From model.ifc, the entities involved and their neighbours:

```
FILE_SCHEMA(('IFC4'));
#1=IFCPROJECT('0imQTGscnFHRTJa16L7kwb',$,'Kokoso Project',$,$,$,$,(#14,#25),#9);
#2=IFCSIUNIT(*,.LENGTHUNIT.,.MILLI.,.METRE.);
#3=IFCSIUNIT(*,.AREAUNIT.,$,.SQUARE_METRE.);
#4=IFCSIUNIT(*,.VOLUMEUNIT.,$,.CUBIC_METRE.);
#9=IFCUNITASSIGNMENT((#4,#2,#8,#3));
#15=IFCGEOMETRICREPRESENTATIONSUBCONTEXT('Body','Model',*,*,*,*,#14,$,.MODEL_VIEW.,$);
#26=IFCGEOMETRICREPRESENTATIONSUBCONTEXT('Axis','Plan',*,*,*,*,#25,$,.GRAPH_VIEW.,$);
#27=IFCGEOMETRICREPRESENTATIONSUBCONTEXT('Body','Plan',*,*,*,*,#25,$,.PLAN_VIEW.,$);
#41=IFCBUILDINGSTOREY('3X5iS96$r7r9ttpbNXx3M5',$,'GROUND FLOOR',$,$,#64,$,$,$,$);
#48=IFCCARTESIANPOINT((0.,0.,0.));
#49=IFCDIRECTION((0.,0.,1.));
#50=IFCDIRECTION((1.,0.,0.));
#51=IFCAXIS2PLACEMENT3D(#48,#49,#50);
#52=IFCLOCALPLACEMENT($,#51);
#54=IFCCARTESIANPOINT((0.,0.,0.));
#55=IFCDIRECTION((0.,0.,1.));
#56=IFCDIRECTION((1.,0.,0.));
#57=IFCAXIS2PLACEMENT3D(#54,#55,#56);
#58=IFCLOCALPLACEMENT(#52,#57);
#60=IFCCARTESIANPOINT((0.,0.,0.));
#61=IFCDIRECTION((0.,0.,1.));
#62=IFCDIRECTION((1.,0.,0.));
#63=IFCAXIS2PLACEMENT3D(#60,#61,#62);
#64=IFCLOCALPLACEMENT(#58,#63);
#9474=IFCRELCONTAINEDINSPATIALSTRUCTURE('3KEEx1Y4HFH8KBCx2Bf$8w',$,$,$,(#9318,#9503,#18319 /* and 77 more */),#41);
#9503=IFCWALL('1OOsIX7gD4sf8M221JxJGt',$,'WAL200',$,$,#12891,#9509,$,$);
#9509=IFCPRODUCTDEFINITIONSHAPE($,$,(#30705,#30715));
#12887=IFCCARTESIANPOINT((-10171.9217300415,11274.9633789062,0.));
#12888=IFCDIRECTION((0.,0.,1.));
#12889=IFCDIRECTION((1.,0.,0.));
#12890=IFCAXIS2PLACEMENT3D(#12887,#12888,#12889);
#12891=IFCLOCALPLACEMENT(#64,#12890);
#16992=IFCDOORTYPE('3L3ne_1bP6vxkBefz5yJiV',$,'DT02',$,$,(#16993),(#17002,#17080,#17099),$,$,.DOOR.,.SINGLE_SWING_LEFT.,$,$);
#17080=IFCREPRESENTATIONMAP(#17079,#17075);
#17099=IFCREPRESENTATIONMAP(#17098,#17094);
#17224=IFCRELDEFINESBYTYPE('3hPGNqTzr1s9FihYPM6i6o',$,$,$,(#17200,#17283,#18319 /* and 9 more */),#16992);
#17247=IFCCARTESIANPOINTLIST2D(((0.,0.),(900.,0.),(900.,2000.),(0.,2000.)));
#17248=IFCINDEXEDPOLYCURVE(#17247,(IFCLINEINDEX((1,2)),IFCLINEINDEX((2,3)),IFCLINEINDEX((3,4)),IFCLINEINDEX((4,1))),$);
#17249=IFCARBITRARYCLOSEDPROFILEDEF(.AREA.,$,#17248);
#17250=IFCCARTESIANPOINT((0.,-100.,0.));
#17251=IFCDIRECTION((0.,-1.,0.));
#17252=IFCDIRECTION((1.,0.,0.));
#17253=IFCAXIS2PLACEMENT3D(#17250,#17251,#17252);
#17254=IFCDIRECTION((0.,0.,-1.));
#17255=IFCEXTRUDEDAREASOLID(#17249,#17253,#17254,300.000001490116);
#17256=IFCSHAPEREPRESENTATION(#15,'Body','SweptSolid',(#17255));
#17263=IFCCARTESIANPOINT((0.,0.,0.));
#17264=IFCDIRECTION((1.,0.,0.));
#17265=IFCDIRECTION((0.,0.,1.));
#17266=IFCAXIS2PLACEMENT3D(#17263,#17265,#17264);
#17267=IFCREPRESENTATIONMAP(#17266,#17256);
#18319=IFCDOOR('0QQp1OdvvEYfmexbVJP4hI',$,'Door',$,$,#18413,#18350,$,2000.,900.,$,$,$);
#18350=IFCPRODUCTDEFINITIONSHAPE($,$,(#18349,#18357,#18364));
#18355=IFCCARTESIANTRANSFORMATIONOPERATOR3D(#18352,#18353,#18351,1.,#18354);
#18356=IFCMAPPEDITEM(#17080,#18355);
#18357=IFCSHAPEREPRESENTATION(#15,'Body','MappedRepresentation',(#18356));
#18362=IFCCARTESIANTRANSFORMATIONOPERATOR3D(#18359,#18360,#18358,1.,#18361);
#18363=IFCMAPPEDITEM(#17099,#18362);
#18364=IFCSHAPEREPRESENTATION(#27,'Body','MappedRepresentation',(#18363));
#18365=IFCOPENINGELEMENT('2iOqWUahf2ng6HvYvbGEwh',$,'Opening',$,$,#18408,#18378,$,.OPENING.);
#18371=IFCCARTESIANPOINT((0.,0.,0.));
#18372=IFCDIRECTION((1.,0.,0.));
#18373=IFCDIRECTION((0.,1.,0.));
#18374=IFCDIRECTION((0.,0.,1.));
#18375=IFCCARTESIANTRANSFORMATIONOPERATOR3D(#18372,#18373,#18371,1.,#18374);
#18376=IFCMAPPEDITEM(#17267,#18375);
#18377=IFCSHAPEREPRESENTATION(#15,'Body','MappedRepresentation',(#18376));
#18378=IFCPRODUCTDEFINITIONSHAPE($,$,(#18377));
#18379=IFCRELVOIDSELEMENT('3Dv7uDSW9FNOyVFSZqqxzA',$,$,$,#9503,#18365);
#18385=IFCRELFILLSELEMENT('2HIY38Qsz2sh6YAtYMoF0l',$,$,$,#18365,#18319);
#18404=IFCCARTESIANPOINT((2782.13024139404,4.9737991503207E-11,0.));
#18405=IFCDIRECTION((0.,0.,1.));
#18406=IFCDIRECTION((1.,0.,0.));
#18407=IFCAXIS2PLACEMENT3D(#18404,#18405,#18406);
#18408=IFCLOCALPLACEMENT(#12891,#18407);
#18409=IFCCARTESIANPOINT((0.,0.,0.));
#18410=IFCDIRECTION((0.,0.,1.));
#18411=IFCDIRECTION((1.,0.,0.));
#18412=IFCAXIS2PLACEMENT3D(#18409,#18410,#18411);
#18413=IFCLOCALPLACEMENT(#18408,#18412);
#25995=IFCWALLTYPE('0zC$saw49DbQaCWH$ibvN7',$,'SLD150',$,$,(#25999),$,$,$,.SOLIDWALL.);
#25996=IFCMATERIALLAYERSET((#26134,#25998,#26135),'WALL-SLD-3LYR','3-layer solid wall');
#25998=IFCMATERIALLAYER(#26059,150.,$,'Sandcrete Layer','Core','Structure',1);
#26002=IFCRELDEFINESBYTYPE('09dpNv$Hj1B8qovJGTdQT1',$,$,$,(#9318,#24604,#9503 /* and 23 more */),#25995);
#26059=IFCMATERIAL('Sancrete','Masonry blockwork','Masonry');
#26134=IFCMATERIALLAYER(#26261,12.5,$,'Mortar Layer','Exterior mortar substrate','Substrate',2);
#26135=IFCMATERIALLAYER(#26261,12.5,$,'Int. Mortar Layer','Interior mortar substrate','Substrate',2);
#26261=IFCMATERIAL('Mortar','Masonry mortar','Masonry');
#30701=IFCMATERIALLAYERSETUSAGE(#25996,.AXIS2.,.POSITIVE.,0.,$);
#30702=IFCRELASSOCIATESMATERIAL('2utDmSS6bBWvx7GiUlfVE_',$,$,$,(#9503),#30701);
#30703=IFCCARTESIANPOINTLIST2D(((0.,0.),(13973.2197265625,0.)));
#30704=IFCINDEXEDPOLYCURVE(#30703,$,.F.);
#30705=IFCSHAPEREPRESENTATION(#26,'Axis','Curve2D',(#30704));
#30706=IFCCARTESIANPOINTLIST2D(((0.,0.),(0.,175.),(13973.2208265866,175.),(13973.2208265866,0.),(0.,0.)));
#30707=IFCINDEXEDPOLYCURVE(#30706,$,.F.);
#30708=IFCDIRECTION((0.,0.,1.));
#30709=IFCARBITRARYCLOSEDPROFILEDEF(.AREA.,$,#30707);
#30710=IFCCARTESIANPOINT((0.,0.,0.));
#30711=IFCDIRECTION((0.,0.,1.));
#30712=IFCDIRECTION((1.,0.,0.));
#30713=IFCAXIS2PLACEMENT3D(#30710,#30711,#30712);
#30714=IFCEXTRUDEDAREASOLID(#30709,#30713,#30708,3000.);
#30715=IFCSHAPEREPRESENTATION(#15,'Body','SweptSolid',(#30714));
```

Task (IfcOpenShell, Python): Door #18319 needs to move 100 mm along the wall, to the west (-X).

```python
import ifcopenshell
import ifcopenshell.api.geometry
import ifcopenshell.util.placement
import ifcopenshell.util.unit

model = ifcopenshell.open("model.ifc")
unit_scale = ifcopenshell.util.unit.calculate_unit_scale(model)

door = model.by_guid("0QQp1OdvvEYfmexbVJP4hI")
opening = door.FillsVoids[0].RelatingOpeningElement
wall = opening.VoidsElements[0].RelatingBuildingElement

wall_matrix = ifcopenshell.util.placement.get_local_placement(wall.ObjectPlacement)
shift = wall_matrix[:3, 0] * -0.1 / unit_scale
before = ifcopenshell.util.placement.get_local_placement(door.ObjectPlacement)[:3, 3].copy()

# The door is placed relative to its opening, so it follows when the opening moves.
matrix = ifcopenshell.util.placement.get_local_placement(opening.ObjectPlacement)
matrix[:3, 3] += shift
ifcopenshell.api.geometry.edit_object_placement(
    model, product=opening, matrix=matrix, is_si=False, should_transform_children=True
)

after = ifcopenshell.util.placement.get_local_placement(door.ObjectPlacement)[:3, 3]
print("door moved by", (after - before).round(3) + 0.0)

model.write("model_updated.ifc")
```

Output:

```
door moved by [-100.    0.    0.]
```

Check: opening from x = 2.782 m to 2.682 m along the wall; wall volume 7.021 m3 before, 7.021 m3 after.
